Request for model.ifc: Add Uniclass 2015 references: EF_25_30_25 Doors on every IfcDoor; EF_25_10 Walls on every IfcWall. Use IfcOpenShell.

First a look at what the model holds.

```python
import ifcopenshell

model = ifcopenshell.open("model.ifc")
print(model.schema)
print("classifications:", [c.Name for c in model.by_type("IfcClassification")])
for ifc_class in ("IfcDoor", "IfcRoof", "IfcStair", "IfcWall", "IfcWindow"):
    print(ifc_class, len(model.by_type(ifc_class)))
```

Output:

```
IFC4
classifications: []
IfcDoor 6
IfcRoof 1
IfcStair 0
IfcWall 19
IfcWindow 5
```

```python
import ifcopenshell
import ifcopenshell.api.classification

model = ifcopenshell.open("model.ifc")

system = ifcopenshell.api.classification.add_classification(model, classification="Uniclass 2015")

codes = {
    "IfcDoor": ("EF_25_30_25", "Doors"),
    "IfcWall": ("EF_25_10", "Walls"),
}
for ifc_class, (code, name) in codes.items():
    products = model.by_type(ifc_class)
    ifcopenshell.api.classification.add_reference(
        model, products=products, classification=system, identification=code, name=name
    )
    print(code, len(products))

model.write("model_rev.ifc")
```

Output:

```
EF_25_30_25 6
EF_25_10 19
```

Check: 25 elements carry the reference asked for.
